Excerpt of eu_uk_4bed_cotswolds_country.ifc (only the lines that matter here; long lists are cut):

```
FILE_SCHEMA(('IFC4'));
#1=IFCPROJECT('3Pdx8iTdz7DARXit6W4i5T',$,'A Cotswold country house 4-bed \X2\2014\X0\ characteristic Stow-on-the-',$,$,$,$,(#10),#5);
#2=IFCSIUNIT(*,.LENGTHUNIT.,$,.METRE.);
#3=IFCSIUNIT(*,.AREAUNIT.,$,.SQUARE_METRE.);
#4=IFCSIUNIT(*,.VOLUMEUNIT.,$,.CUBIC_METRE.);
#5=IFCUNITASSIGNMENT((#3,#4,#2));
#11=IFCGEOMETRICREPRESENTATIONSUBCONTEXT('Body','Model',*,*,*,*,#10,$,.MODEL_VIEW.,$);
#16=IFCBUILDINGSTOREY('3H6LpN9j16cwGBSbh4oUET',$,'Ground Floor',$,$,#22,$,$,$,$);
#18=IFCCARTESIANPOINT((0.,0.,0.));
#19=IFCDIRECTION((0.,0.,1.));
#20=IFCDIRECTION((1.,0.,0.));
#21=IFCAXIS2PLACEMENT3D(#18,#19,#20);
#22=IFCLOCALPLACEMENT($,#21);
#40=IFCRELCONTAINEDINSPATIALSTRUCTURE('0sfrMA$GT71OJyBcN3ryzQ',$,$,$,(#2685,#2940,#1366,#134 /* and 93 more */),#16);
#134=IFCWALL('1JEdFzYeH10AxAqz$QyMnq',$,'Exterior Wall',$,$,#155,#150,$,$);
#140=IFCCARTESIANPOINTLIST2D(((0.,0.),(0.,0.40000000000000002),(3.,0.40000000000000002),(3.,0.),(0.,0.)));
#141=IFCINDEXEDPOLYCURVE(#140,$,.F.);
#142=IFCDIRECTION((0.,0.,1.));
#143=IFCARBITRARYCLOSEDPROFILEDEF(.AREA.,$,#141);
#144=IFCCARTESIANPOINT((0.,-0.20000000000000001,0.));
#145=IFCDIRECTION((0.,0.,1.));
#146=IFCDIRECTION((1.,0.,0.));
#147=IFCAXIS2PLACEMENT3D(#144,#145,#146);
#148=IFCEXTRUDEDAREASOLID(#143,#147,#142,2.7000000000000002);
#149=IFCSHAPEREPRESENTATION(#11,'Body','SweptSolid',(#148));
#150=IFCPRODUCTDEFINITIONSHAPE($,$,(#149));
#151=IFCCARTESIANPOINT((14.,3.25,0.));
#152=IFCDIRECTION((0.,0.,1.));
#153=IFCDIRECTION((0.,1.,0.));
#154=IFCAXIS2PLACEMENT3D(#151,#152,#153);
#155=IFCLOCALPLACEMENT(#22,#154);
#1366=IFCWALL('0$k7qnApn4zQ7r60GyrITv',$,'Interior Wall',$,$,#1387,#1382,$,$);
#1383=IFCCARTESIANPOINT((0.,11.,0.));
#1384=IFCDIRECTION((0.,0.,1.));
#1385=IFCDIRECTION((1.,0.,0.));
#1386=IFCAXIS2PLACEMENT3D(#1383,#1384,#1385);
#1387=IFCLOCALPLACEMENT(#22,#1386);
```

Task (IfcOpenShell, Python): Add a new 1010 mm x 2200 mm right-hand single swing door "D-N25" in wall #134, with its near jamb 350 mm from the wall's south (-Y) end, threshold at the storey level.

```python
import numpy as np
import ifcopenshell
import ifcopenshell.api.feature
import ifcopenshell.api.geometry
import ifcopenshell.api.root
import ifcopenshell.api.spatial
import ifcopenshell.geom
import ifcopenshell.util.element
import ifcopenshell.util.placement
import ifcopenshell.util.representation
import ifcopenshell.util.shape
import ifcopenshell.util.unit

model = ifcopenshell.open("eu_uk_4bed_cotswolds_country.ifc")
unit_scale = ifcopenshell.util.unit.calculate_unit_scale(model)
settings = ifcopenshell.geom.settings()


def volume(element):
    """Net volume in cubic metres, openings subtracted."""
    shape = ifcopenshell.geom.create_shape(settings, element)
    return ifcopenshell.util.shape.get_volume(shape.geometry)


wall = model.by_guid("1JEdFzYeH10AxAqz$QyMnq")
storey = ifcopenshell.util.element.get_container(wall, ifc_class="IfcBuildingStorey")
context = ifcopenshell.util.representation.get_context(model, "Model", "Body", "MODEL_VIEW")
before = volume(wall)

width, height, from_end, sill = 1.01, 2.2, 0.35, 0.0  # metres

# The wall runs along its own X axis, and the end named is its -X end.
wall_shape = ifcopenshell.geom.create_shape(settings, wall)
x, y, z = ifcopenshell.util.shape.get_vertices(wall_shape.geometry).T
start = x.min() + from_end
face, thickness = float(y.min()), float(y.max() - y.min())
wall_matrix = ifcopenshell.util.placement.get_local_placement(wall.ObjectPlacement)
level = ifcopenshell.util.placement.get_local_placement(storey.ObjectPlacement)[2, 3]


def in_wall(x, y):
    """Placement at x, y metres in the wall's axes, at sill height."""
    matrix = wall_matrix.copy()
    matrix[:, 3] = wall_matrix @ np.array([x / unit_scale, y / unit_scale, 0.0, 1.0])
    matrix[2, 3] = level + sill / unit_scale
    return matrix


# Opening: a box that overshoots both wall faces by 50 mm.
opening = ifcopenshell.api.root.create_entity(model, ifc_class="IfcOpeningElement", predefined_type="OPENING")
box = ifcopenshell.api.geometry.add_wall_representation(
    model, context=context, length=width, height=height, thickness=thickness + 0.1
)
ifcopenshell.api.geometry.assign_representation(model, product=opening, representation=box)
ifcopenshell.api.geometry.edit_object_placement(model, product=opening, matrix=in_wall(start, face - 0.05), is_si=False)
ifcopenshell.api.feature.add_feature(model, feature=opening, element=wall)

door = ifcopenshell.api.root.create_entity(model, ifc_class="IfcDoor", name="D-N25", predefined_type="DOOR")
door.OverallWidth, door.OverallHeight = width / unit_scale, height / unit_scale
door.OperationType = "SINGLE_SWING_RIGHT"
body = ifcopenshell.api.geometry.add_door_representation(
    model,
    context=context,
    overall_width=door.OverallWidth,
    overall_height=door.OverallHeight,
    operation_type="SINGLE_SWING_RIGHT",
    lining_properties={"LiningDepth": thickness / unit_scale, "ThresholdDepth": thickness / unit_scale},
)
ifcopenshell.api.geometry.assign_representation(model, product=door, representation=body)
ifcopenshell.api.spatial.assign_container(model, products=[door], relating_structure=storey)
ifcopenshell.api.feature.add_filling(model, opening=opening, element=door)

# The lining spans the wall, so the door starts at the wall face.
ifcopenshell.api.geometry.edit_object_placement(model, product=door, matrix=in_wall(start, face), is_si=False)

after = volume(wall)

print(f"wall volume {before:.3f} -> {after:.3f} m3")

model.write("eu_uk_4bed_cotswolds_country-out.ifc")
```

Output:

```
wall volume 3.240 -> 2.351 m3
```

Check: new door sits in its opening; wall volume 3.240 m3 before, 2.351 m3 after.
